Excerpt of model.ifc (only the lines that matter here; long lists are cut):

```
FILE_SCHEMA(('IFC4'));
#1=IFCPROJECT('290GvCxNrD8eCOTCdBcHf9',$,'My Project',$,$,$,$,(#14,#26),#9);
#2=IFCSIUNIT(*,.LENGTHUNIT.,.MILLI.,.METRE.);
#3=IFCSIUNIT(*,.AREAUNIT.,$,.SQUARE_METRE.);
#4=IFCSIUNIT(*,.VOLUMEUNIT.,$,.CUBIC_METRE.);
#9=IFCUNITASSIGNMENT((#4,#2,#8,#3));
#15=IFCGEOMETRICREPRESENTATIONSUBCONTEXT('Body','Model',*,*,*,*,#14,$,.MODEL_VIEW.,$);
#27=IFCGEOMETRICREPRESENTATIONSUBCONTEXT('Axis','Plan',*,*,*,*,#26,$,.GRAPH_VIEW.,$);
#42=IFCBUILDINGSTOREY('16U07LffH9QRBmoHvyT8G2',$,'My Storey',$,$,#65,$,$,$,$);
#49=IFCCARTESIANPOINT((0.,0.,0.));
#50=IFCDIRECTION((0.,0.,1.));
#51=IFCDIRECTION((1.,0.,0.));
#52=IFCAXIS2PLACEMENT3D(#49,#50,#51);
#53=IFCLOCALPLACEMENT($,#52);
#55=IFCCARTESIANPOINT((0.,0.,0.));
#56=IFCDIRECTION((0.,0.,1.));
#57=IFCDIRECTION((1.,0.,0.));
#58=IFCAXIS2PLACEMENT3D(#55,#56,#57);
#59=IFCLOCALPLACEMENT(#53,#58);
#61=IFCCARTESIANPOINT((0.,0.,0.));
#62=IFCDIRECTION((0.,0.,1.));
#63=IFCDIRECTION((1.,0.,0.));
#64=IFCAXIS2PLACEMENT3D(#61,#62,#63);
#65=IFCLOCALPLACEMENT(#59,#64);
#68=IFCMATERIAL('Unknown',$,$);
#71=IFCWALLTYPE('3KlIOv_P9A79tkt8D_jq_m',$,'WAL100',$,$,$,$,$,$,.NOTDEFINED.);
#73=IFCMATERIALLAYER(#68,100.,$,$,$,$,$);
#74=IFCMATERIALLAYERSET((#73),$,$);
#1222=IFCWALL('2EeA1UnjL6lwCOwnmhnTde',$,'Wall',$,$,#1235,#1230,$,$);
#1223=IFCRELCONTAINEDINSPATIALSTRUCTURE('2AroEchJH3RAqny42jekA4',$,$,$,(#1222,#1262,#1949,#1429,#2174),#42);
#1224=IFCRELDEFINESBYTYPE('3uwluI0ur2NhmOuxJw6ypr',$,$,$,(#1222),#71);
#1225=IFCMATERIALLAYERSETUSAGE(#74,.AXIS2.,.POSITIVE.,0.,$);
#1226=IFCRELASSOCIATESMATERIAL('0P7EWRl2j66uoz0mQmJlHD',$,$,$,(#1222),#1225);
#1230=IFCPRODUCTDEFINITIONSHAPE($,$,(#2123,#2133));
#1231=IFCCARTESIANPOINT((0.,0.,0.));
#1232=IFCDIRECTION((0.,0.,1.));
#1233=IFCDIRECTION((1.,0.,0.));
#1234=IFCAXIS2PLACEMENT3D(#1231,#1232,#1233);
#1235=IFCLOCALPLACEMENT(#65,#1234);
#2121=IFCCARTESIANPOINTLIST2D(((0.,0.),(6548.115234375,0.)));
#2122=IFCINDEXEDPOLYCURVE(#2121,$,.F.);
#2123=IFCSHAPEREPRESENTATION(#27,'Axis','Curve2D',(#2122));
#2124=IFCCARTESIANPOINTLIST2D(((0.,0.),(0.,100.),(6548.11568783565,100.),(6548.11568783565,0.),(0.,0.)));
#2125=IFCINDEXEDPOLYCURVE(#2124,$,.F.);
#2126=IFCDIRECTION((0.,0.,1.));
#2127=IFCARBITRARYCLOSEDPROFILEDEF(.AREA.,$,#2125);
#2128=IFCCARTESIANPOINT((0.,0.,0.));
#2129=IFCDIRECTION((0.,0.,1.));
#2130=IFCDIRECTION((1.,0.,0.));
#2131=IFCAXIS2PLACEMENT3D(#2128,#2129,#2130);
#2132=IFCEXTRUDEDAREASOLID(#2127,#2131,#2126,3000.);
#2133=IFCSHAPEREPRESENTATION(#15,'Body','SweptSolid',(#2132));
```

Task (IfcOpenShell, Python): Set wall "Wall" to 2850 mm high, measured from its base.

```python
import ifcopenshell
import ifcopenshell.geom
import ifcopenshell.util.representation
import ifcopenshell.util.shape
import ifcopenshell.util.unit

model = ifcopenshell.open("model.ifc")
unit_scale = ifcopenshell.util.unit.calculate_unit_scale(model)
settings = ifcopenshell.geom.settings()


def volume(element):
    """Net volume in cubic metres, openings subtracted."""
    shape = ifcopenshell.geom.create_shape(settings, element)
    return ifcopenshell.util.shape.get_volume(shape.geometry)


wall = model.by_guid("2EeA1UnjL6lwCOwnmhnTde")
before = volume(wall)

body = ifcopenshell.util.representation.get_representation(wall, "Model", "Body")
solid = body.Items[0]
old_height = solid.Depth
solid.Depth = 2.85 / unit_scale
after = volume(wall)

print(f"height {old_height:g} -> {solid.Depth:g}, volume {before:.3f} -> {after:.3f} m3")

model.write("model_edited.ifc")
```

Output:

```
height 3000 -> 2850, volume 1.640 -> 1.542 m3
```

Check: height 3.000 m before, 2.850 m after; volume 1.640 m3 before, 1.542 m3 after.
